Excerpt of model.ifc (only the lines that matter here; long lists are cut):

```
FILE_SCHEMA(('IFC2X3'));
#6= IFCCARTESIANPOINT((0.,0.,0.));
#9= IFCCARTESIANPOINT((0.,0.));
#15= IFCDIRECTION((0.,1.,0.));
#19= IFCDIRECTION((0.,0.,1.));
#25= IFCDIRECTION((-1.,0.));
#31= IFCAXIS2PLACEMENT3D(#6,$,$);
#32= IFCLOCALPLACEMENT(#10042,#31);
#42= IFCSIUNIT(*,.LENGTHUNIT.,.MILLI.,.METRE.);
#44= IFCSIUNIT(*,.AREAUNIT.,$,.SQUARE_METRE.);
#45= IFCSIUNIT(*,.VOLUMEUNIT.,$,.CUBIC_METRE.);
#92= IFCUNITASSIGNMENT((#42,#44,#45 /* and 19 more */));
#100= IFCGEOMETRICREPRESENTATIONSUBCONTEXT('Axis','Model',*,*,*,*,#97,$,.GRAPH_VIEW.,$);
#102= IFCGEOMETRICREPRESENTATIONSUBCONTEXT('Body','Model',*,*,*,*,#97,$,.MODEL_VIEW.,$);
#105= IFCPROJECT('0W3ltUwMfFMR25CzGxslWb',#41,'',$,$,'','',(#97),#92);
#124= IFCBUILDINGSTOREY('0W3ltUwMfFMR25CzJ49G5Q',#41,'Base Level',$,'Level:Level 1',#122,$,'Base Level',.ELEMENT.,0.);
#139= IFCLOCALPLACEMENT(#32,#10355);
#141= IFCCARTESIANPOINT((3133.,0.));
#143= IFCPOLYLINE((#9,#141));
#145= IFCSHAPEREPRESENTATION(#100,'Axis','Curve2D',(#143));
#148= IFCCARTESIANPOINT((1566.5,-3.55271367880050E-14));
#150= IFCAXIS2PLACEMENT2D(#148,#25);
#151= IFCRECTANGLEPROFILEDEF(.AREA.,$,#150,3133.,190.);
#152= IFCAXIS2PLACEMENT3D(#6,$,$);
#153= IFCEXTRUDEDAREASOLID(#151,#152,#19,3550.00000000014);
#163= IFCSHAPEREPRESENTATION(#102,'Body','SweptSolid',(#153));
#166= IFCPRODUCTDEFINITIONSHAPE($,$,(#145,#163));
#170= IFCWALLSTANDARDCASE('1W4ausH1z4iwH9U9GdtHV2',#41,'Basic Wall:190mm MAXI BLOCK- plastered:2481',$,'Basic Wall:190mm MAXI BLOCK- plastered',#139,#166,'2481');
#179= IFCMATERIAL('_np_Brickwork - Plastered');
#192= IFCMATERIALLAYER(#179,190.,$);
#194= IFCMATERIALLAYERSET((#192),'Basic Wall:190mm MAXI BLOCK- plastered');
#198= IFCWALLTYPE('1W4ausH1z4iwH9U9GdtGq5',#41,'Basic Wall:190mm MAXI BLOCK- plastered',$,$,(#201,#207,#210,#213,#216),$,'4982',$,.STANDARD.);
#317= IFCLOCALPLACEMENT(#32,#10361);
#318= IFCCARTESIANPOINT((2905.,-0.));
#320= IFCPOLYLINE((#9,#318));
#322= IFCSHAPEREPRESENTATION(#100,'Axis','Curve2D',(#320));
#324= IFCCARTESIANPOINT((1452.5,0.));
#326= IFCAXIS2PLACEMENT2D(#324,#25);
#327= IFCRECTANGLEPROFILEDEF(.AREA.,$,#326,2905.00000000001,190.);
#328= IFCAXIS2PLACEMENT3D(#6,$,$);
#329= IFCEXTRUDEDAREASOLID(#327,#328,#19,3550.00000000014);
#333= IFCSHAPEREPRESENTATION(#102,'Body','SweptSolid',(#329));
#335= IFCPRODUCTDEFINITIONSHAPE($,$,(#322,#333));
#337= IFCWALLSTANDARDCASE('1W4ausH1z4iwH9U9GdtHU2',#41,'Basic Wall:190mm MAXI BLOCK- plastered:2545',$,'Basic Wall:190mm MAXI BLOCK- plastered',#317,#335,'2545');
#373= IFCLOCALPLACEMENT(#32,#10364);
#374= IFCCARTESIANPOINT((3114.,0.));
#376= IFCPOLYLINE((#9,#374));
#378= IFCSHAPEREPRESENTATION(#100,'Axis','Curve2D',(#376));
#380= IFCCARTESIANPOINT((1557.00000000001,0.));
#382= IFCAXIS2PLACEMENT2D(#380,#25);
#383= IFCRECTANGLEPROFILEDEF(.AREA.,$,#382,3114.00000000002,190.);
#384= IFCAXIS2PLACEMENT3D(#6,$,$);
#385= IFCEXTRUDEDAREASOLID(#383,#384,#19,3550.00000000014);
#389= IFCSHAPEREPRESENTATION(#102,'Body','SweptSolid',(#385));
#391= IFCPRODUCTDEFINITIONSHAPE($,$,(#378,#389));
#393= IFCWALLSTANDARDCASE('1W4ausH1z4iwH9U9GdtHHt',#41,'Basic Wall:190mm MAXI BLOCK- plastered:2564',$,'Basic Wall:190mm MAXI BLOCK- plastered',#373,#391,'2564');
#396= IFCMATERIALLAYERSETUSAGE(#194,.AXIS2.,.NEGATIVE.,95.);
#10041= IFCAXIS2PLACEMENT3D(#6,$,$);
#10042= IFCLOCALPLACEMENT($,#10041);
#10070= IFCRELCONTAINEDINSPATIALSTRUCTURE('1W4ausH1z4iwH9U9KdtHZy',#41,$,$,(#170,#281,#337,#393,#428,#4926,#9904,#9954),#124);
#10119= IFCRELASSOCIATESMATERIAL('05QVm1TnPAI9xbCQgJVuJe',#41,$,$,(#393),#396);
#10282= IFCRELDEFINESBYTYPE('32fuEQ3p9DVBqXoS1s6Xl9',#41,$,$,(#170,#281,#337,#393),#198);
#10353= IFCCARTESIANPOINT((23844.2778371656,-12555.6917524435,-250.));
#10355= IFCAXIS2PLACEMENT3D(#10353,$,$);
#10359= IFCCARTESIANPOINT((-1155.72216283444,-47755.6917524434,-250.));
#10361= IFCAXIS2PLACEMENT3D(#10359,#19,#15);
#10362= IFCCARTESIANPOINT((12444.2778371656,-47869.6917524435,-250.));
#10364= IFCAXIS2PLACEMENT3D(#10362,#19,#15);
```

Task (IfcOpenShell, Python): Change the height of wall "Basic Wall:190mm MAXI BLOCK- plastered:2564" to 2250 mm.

```python
import ifcopenshell
import ifcopenshell.geom
import ifcopenshell.util.representation
import ifcopenshell.util.shape
import ifcopenshell.util.unit

model = ifcopenshell.open("model.ifc")
unit_scale = ifcopenshell.util.unit.calculate_unit_scale(model)
settings = ifcopenshell.geom.settings()


def volume(element):
    """Net volume in cubic metres, openings subtracted."""
    shape = ifcopenshell.geom.create_shape(settings, element)
    return ifcopenshell.util.shape.get_volume(shape.geometry)


wall = model.by_id(393)
before = volume(wall)

body = ifcopenshell.util.representation.get_representation(wall, "Model", "Body")
solid = body.Items[0]
old_height = solid.Depth
solid.Depth = 2.25 / unit_scale
after = volume(wall)

print(f"height {old_height:g} -> {solid.Depth:g}, volume {before:.3f} -> {after:.3f} m3")

model.write("model_updated.ifc")
```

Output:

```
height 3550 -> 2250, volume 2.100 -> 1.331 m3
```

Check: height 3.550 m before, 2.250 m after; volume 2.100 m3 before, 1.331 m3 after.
